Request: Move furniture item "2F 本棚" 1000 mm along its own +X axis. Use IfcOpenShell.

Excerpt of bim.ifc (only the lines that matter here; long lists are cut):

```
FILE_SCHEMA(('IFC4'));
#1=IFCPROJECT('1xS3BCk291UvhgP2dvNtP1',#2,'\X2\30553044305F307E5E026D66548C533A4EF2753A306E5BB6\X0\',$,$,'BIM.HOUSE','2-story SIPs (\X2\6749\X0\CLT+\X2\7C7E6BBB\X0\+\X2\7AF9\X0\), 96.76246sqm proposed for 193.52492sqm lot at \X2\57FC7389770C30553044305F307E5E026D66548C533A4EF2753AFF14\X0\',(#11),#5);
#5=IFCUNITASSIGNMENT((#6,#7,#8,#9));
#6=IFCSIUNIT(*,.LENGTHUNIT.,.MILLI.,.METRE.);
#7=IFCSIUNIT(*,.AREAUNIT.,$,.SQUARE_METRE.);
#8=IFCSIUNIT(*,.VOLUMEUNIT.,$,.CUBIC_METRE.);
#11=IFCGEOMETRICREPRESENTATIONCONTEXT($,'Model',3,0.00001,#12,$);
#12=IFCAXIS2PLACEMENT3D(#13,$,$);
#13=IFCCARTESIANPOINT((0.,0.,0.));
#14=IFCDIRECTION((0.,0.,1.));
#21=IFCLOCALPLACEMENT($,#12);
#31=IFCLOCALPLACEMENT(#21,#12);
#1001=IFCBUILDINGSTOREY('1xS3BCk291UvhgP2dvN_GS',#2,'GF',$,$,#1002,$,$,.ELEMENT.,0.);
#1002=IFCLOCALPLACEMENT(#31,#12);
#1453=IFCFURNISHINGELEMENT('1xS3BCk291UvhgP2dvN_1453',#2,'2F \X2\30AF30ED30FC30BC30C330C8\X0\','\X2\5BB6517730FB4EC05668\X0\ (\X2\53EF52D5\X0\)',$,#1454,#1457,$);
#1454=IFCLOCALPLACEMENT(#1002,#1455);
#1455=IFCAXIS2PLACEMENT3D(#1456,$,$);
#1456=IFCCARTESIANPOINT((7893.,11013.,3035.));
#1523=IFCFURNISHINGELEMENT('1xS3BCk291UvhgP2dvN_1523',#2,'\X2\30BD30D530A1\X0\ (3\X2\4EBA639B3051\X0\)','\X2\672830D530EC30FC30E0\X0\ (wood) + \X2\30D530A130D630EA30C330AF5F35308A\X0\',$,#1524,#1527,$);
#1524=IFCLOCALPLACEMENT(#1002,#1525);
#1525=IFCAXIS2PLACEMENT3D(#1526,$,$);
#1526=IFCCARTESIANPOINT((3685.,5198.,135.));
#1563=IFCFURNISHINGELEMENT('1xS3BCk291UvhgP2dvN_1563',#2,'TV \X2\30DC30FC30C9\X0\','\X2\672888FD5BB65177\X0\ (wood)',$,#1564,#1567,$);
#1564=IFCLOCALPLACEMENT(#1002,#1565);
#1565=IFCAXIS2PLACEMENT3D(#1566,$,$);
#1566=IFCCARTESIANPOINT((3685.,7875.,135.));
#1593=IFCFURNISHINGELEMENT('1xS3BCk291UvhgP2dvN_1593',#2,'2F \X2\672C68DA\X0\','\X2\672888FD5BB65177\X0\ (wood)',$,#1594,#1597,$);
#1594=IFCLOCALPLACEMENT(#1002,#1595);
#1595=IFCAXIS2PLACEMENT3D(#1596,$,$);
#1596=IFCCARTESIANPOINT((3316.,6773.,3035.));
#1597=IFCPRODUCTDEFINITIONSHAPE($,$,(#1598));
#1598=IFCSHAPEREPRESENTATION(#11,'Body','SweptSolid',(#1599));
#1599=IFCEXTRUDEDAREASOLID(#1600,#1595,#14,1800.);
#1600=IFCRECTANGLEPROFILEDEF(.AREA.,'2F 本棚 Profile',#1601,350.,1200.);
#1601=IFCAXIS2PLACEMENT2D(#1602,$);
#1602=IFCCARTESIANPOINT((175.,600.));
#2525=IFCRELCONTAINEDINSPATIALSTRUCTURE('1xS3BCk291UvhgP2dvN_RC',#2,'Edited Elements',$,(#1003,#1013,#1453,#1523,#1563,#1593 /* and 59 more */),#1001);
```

```python
import ifcopenshell
import ifcopenshell.api.geometry
import ifcopenshell.util.placement
import ifcopenshell.util.unit

model = ifcopenshell.open("bim.ifc")
unit_scale = ifcopenshell.util.unit.calculate_unit_scale(model)

item = model.by_guid("1xS3BCk291UvhgP2dvN_1593")
matrix = ifcopenshell.util.placement.get_local_placement(item.ObjectPlacement)
matrix[:3, 3] += matrix[:3, 0] * 1 / unit_scale
ifcopenshell.api.geometry.edit_object_placement(model, product=item, matrix=matrix, is_si=False)

print(ifcopenshell.util.placement.get_local_placement(item.ObjectPlacement).round(3) + 0.0)

model.write("bim_v2.ifc")
```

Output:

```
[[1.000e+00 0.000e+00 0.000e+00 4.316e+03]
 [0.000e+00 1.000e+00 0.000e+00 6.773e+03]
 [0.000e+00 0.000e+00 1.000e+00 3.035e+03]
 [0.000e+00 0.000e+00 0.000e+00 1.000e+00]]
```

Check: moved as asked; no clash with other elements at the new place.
